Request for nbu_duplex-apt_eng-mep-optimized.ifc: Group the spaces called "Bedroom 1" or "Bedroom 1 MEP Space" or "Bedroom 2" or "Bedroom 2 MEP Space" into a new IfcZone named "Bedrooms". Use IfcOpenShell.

First a look at what the model holds.

```python
import ifcopenshell

model = ifcopenshell.open("nbu_duplex-apt_eng-mep-optimized.ifc")
print(model.schema)
seen = {}
for space in model.by_type("IfcSpace"):
    seen[space.LongName] = seen.get(space.LongName, 0) + 1
for name, count in sorted(seen.items(), key=str):
    print(count, "x", name)
print("zones:", [z.Name for z in model.by_type("IfcZone")][:20])
```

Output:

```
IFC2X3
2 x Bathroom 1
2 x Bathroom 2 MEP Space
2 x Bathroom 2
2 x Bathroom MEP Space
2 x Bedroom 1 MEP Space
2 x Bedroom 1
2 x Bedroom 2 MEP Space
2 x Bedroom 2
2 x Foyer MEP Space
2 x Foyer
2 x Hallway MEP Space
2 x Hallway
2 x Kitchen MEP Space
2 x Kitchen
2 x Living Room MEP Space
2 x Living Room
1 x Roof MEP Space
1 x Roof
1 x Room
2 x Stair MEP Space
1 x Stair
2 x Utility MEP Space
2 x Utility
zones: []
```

```python
import ifcopenshell
import ifcopenshell.api.group
import ifcopenshell.api.root

model = ifcopenshell.open("nbu_duplex-apt_eng-mep-optimized.ifc")

names = {"Bedroom 1", "Bedroom 1 MEP Space", "Bedroom 2", "Bedroom 2 MEP Space"}
spaces = [s for s in model.by_type("IfcSpace") if s.LongName in names]

zone = ifcopenshell.api.root.create_entity(model, ifc_class="IfcZone", name="Bedrooms")
ifcopenshell.api.group.assign_group(model, products=spaces, group=zone)
print(len(spaces), "spaces in", zone.Name)

model.write("nbu_duplex-apt_eng-mep-optimized_updated.ifc")
```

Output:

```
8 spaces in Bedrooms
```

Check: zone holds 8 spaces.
